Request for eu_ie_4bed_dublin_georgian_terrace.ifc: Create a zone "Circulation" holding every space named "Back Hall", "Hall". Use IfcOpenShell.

First a look at what the model holds.

```python
import ifcopenshell

model = ifcopenshell.open("eu_ie_4bed_dublin_georgian_terrace.ifc")
print(model.schema)
seen = {}
for space in model.by_type("IfcSpace"):
    seen[space.LongName] = seen.get(space.LongName, 0) + 1
for name, count in sorted(seen.items(), key=str):
    print(count, "x", name)
print("zones:", [z.Name for z in model.by_type("IfcZone")][:20])
```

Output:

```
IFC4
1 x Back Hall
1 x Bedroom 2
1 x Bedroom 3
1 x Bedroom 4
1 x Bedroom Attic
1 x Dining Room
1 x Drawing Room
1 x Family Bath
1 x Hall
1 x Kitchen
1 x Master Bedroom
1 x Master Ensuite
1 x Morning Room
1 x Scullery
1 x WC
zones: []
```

```python
import ifcopenshell
import ifcopenshell.api.group
import ifcopenshell.api.root

model = ifcopenshell.open("eu_ie_4bed_dublin_georgian_terrace.ifc")

names = {"Back Hall", "Hall"}
spaces = [s for s in model.by_type("IfcSpace") if s.LongName in names]

zone = ifcopenshell.api.root.create_entity(model, ifc_class="IfcZone", name="Circulation")
ifcopenshell.api.group.assign_group(model, products=spaces, group=zone)
print(len(spaces), "spaces in", zone.Name)

model.write("eu_ie_4bed_dublin_georgian_terrace_rev.ifc")
```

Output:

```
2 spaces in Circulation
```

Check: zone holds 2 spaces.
